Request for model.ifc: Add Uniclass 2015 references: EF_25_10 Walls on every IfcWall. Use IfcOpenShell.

First a look at what the model holds.

```python
import ifcopenshell

model = ifcopenshell.open("model.ifc")
print(model.schema)
print("classifications:", [c.Name for c in model.by_type("IfcClassification")])
for ifc_class in ("IfcDoor", "IfcRoof", "IfcStair", "IfcWall", "IfcWindow"):
    print(ifc_class, len(model.by_type(ifc_class)))
```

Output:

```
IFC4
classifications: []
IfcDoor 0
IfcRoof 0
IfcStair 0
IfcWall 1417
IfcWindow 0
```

```python
import ifcopenshell
import ifcopenshell.api.classification

model = ifcopenshell.open("model.ifc")

system = ifcopenshell.api.classification.add_classification(model, classification="Uniclass 2015")

codes = {
    "IfcWall": ("EF_25_10", "Walls"),
}
for ifc_class, (code, name) in codes.items():
    products = model.by_type(ifc_class)
    ifcopenshell.api.classification.add_reference(
        model, products=products, classification=system, identification=code, name=name
    )
    print(code, len(products))

model.write("model_edited.ifc")
```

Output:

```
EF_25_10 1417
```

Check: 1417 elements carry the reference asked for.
